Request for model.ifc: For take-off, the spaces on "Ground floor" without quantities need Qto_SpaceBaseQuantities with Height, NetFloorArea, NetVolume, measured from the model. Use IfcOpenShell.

First a look at what the model holds.

```python
import ifcopenshell
import ifcopenshell.util.element
import ifcopenshell.util.unit

model = ifcopenshell.open("model.ifc")
print(model.schema)
for unit_type in ("LENGTHUNIT", "AREAUNIT", "VOLUMEUNIT"):
    print(unit_type, ifcopenshell.util.unit.calculate_unit_scale(model, unit_type))
storey = next(s for s in model.by_type("IfcBuildingStorey") if s.Name == "Ground floor")
spaces = [e for e in ifcopenshell.util.element.get_decomposition(storey) if e.is_a("IfcSpace")]
for e in sorted(spaces, key=lambda e: e.id()):
    print(e.id(), e.is_a(), e.Name, list(ifcopenshell.util.element.get_psets(e, qtos_only=True)), sep=" | ")
```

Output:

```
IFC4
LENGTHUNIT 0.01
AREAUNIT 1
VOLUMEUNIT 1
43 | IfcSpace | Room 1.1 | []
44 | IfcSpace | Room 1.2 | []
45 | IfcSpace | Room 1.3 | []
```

```python
import ifcopenshell
import ifcopenshell.api.pset
import ifcopenshell.geom
import ifcopenshell.util.element
import ifcopenshell.util.shape
import ifcopenshell.util.unit

model = ifcopenshell.open("model.ifc")
unit_scale = ifcopenshell.util.unit.calculate_unit_scale(model)
area_scale = ifcopenshell.util.unit.calculate_unit_scale(model, "AREAUNIT")
volume_scale = ifcopenshell.util.unit.calculate_unit_scale(model, "VOLUMEUNIT")
settings = ifcopenshell.geom.settings()

storey = next(s for s in model.by_type("IfcBuildingStorey") if s.Name == "Ground floor")
spaces = [e for e in ifcopenshell.util.element.get_decomposition(storey) if e.is_a("IfcSpace")]

for e in sorted(spaces, key=lambda e: e.id()):
    if ifcopenshell.util.element.get_psets(e, qtos_only=True, should_inherit=False):
        continue
    # Geometry comes back in metres, in the element's own axes.
    shape = ifcopenshell.geom.create_shape(settings, e)
    values = {
        "Height": ifcopenshell.util.shape.get_z(shape.geometry) / unit_scale,
        "NetFloorArea": ifcopenshell.util.shape.get_footprint_area(shape.geometry) / area_scale,
        "NetVolume": ifcopenshell.util.shape.get_volume(shape.geometry) / volume_scale,
    }
    qto = ifcopenshell.api.pset.add_qto(model, product=e, name="Qto_SpaceBaseQuantities")
    ifcopenshell.api.pset.edit_qto(model, qto=qto, properties=values)
    print(e.id(), {k: round(v, 3) for k, v in values.items()})

model.write("model_v2.ifc")
```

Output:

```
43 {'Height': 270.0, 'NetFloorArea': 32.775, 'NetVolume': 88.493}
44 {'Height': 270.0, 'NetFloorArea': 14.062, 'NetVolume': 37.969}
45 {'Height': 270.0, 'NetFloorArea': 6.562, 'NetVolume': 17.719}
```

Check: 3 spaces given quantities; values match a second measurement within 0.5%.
